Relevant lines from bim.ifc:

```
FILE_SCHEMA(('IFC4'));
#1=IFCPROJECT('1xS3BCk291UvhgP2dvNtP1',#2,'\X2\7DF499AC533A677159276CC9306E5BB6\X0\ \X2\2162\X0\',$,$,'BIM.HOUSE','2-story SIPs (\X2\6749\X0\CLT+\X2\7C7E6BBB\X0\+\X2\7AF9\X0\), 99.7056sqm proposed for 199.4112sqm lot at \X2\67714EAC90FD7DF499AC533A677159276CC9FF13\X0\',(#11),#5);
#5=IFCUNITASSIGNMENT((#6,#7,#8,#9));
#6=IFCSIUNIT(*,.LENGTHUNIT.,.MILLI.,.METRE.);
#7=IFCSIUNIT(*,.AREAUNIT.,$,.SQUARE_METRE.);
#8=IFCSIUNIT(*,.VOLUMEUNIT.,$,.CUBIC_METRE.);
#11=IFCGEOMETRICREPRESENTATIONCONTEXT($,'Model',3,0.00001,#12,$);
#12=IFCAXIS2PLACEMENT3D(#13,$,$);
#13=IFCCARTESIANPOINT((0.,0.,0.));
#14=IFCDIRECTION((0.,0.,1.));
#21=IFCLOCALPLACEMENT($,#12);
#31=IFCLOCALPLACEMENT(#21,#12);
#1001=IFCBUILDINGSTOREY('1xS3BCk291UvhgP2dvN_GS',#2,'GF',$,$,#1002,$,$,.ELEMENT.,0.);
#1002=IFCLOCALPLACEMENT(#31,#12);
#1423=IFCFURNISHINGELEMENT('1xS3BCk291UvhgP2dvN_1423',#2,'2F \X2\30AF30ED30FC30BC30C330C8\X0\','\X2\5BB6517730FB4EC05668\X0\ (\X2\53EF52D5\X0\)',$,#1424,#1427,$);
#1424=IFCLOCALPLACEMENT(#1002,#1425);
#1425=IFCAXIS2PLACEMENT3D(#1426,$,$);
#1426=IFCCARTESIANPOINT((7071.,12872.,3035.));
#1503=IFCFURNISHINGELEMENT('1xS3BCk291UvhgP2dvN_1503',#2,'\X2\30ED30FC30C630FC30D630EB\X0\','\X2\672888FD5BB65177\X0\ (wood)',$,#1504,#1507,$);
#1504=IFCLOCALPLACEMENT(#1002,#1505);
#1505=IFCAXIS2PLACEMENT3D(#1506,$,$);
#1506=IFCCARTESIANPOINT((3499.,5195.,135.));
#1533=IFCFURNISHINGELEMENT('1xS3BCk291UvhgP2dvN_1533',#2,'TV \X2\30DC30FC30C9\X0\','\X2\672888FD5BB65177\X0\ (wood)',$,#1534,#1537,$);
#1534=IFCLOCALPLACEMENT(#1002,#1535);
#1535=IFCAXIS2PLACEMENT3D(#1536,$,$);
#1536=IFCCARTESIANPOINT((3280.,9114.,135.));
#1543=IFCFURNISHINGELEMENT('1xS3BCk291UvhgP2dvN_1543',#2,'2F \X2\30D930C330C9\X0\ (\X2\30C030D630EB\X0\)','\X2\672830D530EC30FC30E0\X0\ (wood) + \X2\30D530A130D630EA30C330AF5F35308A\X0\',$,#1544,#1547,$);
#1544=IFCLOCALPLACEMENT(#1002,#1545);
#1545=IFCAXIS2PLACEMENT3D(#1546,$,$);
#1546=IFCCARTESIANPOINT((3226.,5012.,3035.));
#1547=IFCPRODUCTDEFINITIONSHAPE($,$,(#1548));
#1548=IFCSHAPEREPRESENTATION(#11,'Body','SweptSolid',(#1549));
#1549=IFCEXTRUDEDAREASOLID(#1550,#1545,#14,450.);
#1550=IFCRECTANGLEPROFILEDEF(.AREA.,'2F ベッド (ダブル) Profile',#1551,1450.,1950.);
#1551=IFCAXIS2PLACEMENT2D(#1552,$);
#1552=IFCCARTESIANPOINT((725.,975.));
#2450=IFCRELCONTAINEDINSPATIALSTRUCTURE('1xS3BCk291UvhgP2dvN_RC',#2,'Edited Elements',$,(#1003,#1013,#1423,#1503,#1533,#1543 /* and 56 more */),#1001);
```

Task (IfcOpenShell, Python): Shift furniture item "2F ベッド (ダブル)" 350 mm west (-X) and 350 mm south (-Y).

```python
import ifcopenshell
import ifcopenshell.api.geometry
import ifcopenshell.util.placement

model = ifcopenshell.open("bim.ifc")

item = model.by_guid("1xS3BCk291UvhgP2dvN_1543")
matrix = ifcopenshell.util.placement.get_local_placement(item.ObjectPlacement)
matrix[0, 3] -= 350.0
matrix[1, 3] -= 350.0
ifcopenshell.api.geometry.edit_object_placement(model, product=item, matrix=matrix, is_si=False)

print(ifcopenshell.util.placement.get_local_placement(item.ObjectPlacement).round(3) + 0.0)

model.write("bim_v2.ifc")
```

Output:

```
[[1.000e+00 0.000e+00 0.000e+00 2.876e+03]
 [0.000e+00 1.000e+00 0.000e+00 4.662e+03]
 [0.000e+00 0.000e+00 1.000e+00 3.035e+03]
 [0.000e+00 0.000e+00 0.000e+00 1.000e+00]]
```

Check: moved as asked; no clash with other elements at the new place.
